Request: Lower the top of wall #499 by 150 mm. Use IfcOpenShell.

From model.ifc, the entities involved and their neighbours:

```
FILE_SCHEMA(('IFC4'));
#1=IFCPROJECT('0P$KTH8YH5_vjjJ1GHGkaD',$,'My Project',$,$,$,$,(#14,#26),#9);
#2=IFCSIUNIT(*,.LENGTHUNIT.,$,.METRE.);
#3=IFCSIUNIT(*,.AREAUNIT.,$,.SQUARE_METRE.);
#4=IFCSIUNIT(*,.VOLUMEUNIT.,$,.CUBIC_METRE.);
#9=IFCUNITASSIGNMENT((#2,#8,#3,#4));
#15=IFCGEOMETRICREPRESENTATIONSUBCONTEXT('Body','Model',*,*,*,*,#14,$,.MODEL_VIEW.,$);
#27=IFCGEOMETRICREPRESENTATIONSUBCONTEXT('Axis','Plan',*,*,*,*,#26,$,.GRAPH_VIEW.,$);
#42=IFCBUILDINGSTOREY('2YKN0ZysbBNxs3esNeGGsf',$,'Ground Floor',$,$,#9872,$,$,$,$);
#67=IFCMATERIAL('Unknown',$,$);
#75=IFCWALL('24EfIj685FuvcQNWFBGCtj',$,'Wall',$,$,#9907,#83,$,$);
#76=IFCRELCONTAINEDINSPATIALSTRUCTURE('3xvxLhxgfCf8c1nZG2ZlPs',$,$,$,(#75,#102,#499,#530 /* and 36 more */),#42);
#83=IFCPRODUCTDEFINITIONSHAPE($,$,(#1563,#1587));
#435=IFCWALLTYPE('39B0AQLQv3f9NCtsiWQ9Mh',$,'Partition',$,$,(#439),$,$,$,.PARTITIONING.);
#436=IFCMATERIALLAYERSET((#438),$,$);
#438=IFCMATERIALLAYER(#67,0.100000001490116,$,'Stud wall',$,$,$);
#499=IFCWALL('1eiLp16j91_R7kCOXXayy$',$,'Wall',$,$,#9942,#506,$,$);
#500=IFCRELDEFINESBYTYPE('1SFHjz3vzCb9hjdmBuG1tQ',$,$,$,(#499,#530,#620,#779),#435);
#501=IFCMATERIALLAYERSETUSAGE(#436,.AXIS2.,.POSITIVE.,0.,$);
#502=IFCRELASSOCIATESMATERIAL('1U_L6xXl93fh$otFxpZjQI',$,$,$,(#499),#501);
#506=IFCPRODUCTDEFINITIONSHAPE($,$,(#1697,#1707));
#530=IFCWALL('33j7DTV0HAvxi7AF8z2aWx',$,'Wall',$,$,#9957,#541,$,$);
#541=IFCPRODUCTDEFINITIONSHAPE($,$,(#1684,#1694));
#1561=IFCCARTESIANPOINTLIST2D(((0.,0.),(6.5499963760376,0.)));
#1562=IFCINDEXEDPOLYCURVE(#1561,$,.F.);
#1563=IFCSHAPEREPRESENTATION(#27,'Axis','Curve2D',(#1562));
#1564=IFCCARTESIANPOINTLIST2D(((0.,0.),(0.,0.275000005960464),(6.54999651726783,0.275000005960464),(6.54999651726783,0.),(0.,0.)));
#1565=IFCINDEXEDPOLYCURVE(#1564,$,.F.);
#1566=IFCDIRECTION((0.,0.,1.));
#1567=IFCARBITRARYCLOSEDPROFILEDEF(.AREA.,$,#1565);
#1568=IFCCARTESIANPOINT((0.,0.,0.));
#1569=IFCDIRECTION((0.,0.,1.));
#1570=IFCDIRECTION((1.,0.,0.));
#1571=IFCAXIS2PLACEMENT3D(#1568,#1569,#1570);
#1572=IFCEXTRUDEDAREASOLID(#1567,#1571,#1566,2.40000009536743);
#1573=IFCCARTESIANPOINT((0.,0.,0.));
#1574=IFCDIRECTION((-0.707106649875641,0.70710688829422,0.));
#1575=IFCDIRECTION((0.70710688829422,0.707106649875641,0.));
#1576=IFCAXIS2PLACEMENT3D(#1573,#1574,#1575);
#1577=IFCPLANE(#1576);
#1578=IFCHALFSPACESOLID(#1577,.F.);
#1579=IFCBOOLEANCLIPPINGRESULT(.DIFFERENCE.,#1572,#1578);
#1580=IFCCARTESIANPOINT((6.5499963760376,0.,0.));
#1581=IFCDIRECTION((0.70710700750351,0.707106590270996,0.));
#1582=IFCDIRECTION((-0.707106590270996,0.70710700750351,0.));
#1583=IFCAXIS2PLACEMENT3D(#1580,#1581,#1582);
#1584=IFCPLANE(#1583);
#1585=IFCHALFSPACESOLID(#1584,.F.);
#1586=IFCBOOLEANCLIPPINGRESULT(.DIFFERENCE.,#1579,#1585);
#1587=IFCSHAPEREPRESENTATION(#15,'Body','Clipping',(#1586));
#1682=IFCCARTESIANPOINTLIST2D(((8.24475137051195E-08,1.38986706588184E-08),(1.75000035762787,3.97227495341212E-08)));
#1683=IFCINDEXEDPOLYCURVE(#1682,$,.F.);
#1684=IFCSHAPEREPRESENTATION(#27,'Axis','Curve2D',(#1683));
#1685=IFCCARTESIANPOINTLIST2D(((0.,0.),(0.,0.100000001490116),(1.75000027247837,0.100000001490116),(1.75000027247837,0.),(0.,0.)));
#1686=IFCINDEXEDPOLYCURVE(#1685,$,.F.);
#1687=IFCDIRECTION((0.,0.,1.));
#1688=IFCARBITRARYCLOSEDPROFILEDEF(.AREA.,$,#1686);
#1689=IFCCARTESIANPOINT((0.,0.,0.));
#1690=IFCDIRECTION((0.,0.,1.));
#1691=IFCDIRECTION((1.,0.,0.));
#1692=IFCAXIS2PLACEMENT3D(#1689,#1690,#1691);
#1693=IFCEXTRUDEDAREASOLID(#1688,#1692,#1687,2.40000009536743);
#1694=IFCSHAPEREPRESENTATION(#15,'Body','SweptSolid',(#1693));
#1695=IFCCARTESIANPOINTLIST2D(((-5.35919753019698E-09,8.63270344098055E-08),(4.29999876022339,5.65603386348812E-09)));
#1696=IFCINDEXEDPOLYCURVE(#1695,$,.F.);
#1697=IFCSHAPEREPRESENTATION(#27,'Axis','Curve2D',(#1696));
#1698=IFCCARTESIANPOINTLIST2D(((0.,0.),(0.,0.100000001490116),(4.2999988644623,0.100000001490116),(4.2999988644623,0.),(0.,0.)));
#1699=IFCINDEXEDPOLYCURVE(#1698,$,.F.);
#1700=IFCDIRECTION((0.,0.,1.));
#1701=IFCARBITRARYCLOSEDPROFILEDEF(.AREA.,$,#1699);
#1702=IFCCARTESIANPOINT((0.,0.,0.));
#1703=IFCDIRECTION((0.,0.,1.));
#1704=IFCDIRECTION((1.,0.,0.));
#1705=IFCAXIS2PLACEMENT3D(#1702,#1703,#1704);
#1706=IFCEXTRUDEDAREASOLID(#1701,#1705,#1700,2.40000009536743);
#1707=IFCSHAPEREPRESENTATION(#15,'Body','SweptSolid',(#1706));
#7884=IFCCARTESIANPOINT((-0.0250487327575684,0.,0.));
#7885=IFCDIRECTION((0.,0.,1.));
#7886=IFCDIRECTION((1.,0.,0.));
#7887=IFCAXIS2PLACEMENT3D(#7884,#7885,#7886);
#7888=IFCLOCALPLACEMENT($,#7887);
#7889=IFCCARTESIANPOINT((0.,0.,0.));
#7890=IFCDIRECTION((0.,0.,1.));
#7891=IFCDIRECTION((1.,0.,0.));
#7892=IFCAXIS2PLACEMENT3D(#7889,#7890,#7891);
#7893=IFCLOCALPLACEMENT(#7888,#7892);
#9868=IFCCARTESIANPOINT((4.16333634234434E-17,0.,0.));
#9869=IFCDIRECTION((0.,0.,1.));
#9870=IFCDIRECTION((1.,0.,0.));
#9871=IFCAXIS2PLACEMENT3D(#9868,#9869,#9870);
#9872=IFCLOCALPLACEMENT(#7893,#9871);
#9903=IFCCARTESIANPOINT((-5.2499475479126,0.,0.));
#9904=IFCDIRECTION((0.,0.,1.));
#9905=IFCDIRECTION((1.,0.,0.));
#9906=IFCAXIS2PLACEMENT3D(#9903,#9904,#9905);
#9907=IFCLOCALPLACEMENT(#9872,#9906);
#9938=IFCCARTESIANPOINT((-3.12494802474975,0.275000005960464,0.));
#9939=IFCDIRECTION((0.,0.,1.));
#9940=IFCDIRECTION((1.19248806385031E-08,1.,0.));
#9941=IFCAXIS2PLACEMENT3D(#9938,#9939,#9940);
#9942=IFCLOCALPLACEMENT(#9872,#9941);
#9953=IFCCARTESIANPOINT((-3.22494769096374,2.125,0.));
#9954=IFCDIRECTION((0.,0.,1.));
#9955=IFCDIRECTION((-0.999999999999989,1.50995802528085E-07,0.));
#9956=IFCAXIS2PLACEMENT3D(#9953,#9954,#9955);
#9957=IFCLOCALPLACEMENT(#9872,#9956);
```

```python
import ifcopenshell
import ifcopenshell.geom
import ifcopenshell.util.representation
import ifcopenshell.util.shape
import ifcopenshell.util.unit

model = ifcopenshell.open("model.ifc")
unit_scale = ifcopenshell.util.unit.calculate_unit_scale(model)
settings = ifcopenshell.geom.settings()


def volume(element):
    """Net volume in cubic metres, openings subtracted."""
    shape = ifcopenshell.geom.create_shape(settings, element)
    return ifcopenshell.util.shape.get_volume(shape.geometry)


wall = model.by_id(499)
before = volume(wall)

body = ifcopenshell.util.representation.get_representation(wall, "Model", "Body")
solid = body.Items[0]
old_height = solid.Depth
solid.Depth -= 0.15 / unit_scale
after = volume(wall)

print(f"height {old_height:g} -> {solid.Depth:g}, volume {before:.3f} -> {after:.3f} m3")

model.write("model_updated.ifc")
```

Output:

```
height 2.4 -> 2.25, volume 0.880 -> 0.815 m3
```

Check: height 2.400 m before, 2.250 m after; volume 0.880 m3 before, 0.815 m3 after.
